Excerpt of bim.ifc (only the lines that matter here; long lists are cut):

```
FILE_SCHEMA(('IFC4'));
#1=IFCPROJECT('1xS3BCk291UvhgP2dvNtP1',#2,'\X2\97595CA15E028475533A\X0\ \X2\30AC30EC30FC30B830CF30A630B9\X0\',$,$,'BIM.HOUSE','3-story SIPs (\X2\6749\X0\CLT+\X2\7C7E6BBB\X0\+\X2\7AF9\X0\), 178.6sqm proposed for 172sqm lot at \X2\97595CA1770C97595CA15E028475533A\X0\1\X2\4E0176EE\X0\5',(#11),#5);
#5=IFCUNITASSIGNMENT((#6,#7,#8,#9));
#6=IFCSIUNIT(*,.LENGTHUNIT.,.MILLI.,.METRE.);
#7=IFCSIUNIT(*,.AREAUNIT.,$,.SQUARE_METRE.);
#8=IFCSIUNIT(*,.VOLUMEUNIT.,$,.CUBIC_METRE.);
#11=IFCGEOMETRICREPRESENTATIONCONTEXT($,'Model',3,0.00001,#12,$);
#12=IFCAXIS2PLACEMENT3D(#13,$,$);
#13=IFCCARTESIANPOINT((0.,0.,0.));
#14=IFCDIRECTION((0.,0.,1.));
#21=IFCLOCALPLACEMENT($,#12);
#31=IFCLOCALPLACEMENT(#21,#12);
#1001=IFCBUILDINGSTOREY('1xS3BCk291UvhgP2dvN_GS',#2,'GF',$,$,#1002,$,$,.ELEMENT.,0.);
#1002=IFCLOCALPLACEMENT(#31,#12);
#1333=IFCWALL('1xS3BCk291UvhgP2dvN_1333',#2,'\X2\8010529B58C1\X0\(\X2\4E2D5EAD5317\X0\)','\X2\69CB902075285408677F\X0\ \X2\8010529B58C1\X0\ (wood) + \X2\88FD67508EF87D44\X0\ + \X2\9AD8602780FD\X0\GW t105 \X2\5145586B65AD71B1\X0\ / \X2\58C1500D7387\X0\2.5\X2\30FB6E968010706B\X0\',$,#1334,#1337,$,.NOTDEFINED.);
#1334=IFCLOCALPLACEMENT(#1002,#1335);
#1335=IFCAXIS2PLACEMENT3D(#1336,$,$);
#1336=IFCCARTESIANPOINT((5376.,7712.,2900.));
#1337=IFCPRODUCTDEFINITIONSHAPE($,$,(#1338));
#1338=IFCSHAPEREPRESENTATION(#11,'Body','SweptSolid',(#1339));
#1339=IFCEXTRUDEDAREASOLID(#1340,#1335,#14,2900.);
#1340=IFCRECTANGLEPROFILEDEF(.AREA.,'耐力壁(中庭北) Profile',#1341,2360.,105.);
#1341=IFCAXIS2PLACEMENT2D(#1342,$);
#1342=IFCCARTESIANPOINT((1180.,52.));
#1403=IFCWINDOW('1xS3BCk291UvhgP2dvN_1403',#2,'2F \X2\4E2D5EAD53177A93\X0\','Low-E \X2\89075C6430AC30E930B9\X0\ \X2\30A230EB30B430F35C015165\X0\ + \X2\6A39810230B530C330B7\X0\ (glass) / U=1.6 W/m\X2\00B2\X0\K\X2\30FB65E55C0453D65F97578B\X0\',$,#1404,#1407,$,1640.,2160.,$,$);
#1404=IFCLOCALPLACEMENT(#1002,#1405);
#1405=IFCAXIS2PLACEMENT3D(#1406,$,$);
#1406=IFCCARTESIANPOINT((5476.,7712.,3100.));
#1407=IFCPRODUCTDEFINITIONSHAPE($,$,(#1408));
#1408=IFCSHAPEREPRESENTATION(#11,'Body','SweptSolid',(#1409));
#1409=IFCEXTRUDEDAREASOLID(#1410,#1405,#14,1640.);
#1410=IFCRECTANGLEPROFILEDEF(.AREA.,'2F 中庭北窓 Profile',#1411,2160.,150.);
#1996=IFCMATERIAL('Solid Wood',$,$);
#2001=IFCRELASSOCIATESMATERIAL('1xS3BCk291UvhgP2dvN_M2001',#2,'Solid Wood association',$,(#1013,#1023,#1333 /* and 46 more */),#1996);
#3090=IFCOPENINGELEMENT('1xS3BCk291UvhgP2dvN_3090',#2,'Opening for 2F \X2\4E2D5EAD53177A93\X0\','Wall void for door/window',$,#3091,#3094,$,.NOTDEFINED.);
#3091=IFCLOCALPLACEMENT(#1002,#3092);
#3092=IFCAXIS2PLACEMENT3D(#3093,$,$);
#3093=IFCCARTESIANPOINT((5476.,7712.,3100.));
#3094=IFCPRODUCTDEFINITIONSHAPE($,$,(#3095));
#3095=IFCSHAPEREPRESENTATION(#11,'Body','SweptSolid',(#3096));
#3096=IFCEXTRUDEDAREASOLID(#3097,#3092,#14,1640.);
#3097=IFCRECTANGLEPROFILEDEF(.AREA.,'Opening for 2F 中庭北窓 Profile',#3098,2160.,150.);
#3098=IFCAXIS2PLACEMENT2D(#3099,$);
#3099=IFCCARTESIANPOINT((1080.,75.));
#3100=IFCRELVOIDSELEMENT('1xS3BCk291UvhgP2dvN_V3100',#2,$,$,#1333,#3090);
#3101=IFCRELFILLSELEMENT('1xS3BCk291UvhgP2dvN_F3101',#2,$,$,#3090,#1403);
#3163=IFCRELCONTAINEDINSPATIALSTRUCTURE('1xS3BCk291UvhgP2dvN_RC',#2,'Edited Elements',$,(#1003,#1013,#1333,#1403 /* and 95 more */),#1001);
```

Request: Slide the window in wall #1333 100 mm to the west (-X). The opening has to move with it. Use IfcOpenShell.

```python
import ifcopenshell
import ifcopenshell.api.geometry
import ifcopenshell.util.placement
import ifcopenshell.util.unit

model = ifcopenshell.open("bim.ifc")
unit_scale = ifcopenshell.util.unit.calculate_unit_scale(model)

window = model.by_id(1403)
opening = window.FillsVoids[0].RelatingOpeningElement
wall = opening.VoidsElements[0].RelatingBuildingElement

wall_matrix = ifcopenshell.util.placement.get_local_placement(wall.ObjectPlacement)
shift = wall_matrix[:3, 0] * -0.1 / unit_scale
before = ifcopenshell.util.placement.get_local_placement(window.ObjectPlacement)[:3, 3].copy()

# The window is not placed relative to its opening, so move both.
for product in (opening, window):
    matrix = ifcopenshell.util.placement.get_local_placement(product.ObjectPlacement)
    matrix[:3, 3] += shift
    ifcopenshell.api.geometry.edit_object_placement(model, product=product, matrix=matrix, is_si=False)

after = ifcopenshell.util.placement.get_local_placement(window.ObjectPlacement)[:3, 3]
print("window moved by", (after - before).round(3) + 0.0)

model.write("bim_updated.ifc")
```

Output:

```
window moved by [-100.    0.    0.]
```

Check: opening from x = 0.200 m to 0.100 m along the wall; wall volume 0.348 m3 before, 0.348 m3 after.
